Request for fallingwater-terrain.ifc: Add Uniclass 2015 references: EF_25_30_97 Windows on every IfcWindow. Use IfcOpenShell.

First a look at what the model holds.

```python
import ifcopenshell

model = ifcopenshell.open("fallingwater-terrain.ifc")
print(model.schema)
print("classifications:", [c.Name for c in model.by_type("IfcClassification")])
for ifc_class in ("IfcDoor", "IfcRoof", "IfcStair", "IfcWall", "IfcWindow"):
    print(ifc_class, len(model.by_type(ifc_class)))
```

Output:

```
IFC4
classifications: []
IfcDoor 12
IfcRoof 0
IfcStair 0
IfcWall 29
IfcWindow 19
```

```python
import ifcopenshell
import ifcopenshell.api.classification

model = ifcopenshell.open("fallingwater-terrain.ifc")

system = ifcopenshell.api.classification.add_classification(model, classification="Uniclass 2015")

codes = {
    "IfcWindow": ("EF_25_30_97", "Windows"),
}
for ifc_class, (code, name) in codes.items():
    products = model.by_type(ifc_class)
    ifcopenshell.api.classification.add_reference(
        model, products=products, classification=system, identification=code, name=name
    )
    print(code, len(products))

model.write("fallingwater-terrain-out.ifc")
```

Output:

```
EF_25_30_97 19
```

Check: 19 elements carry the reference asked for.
